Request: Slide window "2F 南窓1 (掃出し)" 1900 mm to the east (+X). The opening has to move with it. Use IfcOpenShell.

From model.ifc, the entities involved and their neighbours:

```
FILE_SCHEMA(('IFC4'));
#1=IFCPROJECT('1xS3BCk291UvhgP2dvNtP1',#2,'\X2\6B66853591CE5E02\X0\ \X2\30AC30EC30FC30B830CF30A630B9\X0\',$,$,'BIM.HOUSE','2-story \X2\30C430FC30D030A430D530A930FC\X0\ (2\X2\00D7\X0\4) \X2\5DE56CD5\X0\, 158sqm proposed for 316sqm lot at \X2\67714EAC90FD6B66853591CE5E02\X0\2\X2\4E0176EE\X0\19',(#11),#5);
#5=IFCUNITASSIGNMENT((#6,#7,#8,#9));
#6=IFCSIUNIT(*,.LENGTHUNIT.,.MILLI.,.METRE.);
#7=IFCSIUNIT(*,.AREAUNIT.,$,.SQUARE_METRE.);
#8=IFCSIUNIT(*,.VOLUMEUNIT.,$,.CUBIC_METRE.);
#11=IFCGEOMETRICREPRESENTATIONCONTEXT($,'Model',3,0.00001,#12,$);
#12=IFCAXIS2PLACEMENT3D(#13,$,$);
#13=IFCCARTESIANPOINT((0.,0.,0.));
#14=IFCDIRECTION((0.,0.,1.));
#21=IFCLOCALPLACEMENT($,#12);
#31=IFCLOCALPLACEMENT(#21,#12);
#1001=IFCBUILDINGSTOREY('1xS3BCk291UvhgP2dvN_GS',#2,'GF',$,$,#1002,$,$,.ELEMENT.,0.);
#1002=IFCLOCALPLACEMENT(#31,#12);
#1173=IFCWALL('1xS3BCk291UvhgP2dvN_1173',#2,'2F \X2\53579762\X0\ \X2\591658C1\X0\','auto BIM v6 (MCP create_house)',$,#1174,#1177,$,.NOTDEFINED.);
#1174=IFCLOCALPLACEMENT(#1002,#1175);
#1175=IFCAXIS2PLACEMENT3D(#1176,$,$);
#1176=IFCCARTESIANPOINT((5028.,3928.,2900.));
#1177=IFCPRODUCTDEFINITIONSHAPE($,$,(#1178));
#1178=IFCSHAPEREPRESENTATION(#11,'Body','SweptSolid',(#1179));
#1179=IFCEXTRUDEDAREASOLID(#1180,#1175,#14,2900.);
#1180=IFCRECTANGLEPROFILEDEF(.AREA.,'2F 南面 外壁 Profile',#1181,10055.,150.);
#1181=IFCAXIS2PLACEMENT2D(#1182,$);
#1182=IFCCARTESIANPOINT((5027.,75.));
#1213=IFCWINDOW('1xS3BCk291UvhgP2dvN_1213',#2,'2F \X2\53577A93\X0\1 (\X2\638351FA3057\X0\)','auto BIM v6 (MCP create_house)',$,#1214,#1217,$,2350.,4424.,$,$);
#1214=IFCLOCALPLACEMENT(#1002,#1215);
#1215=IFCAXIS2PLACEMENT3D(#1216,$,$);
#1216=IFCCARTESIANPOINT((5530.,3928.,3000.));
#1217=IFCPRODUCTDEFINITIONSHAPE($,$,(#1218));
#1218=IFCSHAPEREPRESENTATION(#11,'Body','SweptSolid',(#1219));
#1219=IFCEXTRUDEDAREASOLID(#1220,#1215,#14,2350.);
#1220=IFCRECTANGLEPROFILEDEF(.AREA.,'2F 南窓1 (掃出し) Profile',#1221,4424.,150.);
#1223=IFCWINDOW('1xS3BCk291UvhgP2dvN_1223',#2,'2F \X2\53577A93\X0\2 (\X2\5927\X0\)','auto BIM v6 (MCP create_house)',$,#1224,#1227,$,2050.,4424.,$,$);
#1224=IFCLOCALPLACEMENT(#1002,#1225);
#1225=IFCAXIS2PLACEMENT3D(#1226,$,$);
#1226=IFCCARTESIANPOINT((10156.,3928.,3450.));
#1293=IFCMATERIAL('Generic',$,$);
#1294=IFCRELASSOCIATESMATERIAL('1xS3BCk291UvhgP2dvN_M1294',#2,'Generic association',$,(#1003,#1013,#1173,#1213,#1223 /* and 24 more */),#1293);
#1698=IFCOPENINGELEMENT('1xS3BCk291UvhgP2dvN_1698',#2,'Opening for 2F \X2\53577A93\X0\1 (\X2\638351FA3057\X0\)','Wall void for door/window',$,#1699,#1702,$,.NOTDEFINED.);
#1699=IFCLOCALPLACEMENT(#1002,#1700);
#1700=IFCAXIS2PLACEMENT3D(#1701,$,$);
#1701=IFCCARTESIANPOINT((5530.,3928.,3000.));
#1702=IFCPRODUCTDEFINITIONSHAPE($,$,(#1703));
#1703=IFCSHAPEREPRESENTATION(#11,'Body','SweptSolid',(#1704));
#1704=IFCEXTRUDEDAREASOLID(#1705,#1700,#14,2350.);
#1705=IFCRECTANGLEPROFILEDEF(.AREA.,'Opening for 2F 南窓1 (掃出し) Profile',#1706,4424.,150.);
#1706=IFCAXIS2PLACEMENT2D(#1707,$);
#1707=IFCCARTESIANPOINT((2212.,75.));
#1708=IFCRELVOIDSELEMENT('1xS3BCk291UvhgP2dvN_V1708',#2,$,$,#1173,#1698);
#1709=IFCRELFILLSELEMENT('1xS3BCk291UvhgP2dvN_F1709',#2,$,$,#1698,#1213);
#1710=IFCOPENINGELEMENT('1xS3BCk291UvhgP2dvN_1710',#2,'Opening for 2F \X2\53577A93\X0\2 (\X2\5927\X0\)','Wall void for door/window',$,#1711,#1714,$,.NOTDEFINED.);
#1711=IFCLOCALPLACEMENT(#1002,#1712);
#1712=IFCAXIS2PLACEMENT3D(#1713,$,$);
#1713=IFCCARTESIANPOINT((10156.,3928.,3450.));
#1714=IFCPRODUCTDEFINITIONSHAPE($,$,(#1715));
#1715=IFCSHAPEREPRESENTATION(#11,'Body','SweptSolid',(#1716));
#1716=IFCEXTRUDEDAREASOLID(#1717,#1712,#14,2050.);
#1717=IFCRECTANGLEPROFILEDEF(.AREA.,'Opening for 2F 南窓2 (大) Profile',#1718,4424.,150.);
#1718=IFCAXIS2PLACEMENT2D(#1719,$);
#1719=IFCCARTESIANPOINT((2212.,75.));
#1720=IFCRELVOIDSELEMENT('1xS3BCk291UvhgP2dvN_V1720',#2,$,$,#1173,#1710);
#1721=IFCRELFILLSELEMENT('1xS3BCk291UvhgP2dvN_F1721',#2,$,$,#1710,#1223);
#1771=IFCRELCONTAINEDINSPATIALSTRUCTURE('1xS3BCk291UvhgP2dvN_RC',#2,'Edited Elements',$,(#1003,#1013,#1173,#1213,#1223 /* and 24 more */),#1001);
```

```python
import ifcopenshell
import ifcopenshell.api.geometry
import ifcopenshell.util.placement
import ifcopenshell.util.unit

model = ifcopenshell.open("model.ifc")
unit_scale = ifcopenshell.util.unit.calculate_unit_scale(model)

window = model.by_id(1213)
opening = window.FillsVoids[0].RelatingOpeningElement
wall = opening.VoidsElements[0].RelatingBuildingElement

wall_matrix = ifcopenshell.util.placement.get_local_placement(wall.ObjectPlacement)
shift = wall_matrix[:3, 0] * 1.9 / unit_scale
before = ifcopenshell.util.placement.get_local_placement(window.ObjectPlacement)[:3, 3].copy()

# The window is not placed relative to its opening, so move both.
for product in (opening, window):
    matrix = ifcopenshell.util.placement.get_local_placement(product.ObjectPlacement)
    matrix[:3, 3] += shift
    ifcopenshell.api.geometry.edit_object_placement(model, product=product, matrix=matrix, is_si=False)

after = ifcopenshell.util.placement.get_local_placement(window.ObjectPlacement)[:3, 3]
print("window moved by", (after - before).round(3) + 0.0)

model.write("model_v2.ifc")
```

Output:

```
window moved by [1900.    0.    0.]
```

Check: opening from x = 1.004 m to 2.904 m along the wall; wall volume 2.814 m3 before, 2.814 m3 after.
